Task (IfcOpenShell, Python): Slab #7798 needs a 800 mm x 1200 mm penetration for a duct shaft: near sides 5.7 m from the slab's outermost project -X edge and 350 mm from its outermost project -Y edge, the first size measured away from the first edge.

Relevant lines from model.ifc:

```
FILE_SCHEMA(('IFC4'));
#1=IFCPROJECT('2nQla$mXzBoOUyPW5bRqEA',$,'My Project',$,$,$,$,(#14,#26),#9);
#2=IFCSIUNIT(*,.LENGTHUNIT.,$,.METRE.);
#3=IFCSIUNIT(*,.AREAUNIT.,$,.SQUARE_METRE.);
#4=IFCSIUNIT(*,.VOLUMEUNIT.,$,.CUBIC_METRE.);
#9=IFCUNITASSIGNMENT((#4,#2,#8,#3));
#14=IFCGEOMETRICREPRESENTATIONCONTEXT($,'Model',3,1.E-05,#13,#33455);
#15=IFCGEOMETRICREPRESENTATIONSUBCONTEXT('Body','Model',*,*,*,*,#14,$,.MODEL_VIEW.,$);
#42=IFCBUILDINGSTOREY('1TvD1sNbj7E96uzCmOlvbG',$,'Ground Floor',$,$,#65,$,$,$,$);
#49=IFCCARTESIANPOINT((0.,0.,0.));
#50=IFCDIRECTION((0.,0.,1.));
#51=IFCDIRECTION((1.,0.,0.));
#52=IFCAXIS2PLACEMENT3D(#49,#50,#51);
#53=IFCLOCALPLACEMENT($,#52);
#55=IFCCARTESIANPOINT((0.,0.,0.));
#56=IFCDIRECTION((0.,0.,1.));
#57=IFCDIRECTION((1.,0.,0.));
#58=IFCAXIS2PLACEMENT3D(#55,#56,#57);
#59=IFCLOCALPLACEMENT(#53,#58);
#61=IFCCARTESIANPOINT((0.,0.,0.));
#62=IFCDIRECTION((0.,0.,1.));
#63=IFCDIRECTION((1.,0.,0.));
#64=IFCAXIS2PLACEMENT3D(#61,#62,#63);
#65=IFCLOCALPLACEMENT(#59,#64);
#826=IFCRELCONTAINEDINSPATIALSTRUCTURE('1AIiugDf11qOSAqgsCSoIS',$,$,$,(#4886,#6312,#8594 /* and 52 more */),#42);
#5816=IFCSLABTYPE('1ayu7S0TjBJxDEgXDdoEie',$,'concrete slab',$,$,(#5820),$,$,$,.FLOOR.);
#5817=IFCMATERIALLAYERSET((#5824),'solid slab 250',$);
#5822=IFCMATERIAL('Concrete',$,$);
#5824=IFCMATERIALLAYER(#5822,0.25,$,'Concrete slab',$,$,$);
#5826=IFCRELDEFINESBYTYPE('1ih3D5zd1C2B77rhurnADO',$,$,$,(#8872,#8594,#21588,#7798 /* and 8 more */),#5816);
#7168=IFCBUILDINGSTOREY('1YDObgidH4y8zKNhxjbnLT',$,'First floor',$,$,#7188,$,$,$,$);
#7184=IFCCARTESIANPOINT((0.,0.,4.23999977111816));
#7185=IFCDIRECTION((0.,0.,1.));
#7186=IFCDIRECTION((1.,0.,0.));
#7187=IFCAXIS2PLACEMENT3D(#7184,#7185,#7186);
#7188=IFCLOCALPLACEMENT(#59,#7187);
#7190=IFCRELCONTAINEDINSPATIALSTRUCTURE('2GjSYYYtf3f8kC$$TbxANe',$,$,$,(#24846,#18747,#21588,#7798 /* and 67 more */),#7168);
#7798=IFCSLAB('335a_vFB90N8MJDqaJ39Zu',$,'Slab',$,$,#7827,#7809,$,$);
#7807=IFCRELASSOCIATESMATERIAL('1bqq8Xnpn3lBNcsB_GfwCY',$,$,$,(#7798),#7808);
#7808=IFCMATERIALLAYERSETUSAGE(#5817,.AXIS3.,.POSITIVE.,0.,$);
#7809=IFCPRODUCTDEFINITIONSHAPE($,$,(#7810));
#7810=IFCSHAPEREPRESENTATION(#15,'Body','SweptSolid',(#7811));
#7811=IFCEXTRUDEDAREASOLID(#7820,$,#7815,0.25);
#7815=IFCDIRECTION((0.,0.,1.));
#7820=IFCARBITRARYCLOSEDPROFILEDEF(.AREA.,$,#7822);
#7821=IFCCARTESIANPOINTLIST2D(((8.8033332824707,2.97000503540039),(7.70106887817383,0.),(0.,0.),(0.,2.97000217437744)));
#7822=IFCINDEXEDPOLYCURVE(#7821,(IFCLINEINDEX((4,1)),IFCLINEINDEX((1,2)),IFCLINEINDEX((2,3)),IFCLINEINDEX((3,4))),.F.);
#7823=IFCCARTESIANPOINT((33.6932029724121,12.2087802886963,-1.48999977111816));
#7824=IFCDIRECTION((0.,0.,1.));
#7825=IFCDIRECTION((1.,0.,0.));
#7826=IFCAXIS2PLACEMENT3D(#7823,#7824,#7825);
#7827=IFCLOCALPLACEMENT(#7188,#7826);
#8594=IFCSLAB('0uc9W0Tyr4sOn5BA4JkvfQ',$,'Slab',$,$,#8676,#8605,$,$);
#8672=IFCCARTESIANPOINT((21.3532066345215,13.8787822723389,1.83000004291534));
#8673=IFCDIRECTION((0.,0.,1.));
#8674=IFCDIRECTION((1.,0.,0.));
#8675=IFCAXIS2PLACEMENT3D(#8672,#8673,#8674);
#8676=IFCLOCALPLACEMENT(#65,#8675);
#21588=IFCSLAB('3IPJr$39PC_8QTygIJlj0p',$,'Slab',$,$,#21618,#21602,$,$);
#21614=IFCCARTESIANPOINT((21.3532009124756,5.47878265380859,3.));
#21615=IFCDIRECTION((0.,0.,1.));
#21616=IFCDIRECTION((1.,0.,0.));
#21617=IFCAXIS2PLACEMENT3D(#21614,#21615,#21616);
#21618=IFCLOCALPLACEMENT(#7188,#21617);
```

```python
import numpy as np
import ifcopenshell
import ifcopenshell.api.feature
import ifcopenshell.api.geometry
import ifcopenshell.api.root
import ifcopenshell.geom
import ifcopenshell.util.placement
import ifcopenshell.util.representation
import ifcopenshell.util.shape
import ifcopenshell.util.unit

model = ifcopenshell.open("model.ifc")
unit_scale = ifcopenshell.util.unit.calculate_unit_scale(model)
settings = ifcopenshell.geom.settings()


def volume(element):
    """Net volume in cubic metres, openings subtracted."""
    shape = ifcopenshell.geom.create_shape(settings, element)
    return ifcopenshell.util.shape.get_volume(shape.geometry)


slab = model.by_guid("335a_vFB90N8MJDqaJ39Zu")
before = volume(slab)

# Extent in the slab's own axes, in metres. The edges named are its -X and -Y sides.
slab_shape = ifcopenshell.geom.create_shape(settings, slab)
vertices = ifcopenshell.util.shape.get_vertices(slab_shape.geometry)
x_min, y_min, bottom = vertices.min(axis=0)
top = vertices[:, 2].max()

opening = ifcopenshell.api.root.create_entity(model, ifc_class="IfcOpeningElement", name="Duct shaft opening", predefined_type="OPENING")
context = ifcopenshell.util.representation.get_context(model, "Model", "Body", "MODEL_VIEW")
width, depth = 0.8, 1.2
outline = [(0.0, 0.0), (width, 0.0), (width, depth), (0.0, depth), (0.0, 0.0)]
# Overshoot both faces by 50 mm so the cut is clean.
shape = ifcopenshell.api.geometry.add_slab_representation(
    model, context=context, depth=top - bottom + 0.1, polyline=outline
)
ifcopenshell.api.geometry.assign_representation(model, product=opening, representation=shape)

matrix = ifcopenshell.util.placement.get_local_placement(slab.ObjectPlacement)
matrix[:, 3] = matrix @ np.append(np.array([x_min + 5.7, y_min + 0.35, bottom - 0.05]) / unit_scale, 1.0)
ifcopenshell.api.geometry.edit_object_placement(model, product=opening, matrix=matrix, is_si=False)
ifcopenshell.api.feature.add_feature(model, feature=opening, element=slab)

after = volume(slab)

print(f"slab volume {before:.3f} -> {after:.3f} m3")

model.write("model_edited.ifc")
```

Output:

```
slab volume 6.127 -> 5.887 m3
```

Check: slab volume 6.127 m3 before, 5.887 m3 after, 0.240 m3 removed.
